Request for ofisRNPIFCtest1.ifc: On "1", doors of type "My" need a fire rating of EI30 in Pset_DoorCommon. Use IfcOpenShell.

First a look at what the model holds.

```python
import ifcopenshell
import ifcopenshell.util.element

model = ifcopenshell.open("ofisRNPIFCtest1.ifc")
print(model.schema)
storey = next(s for s in model.by_type("IfcBuildingStorey") if s.Name == "1")
doors = [e for e in ifcopenshell.util.element.get_decomposition(storey) if e.is_a("IfcDoor")]
seen = {}
for e in doors:
    element_type = ifcopenshell.util.element.get_type(e)
    key = (element_type.Name if element_type != e and element_type else None, ifcopenshell.util.element.get_pset(e, "Pset_DoorCommon", "FireRating"))
    seen[key] = seen.get(key, 0) + 1
for (name, value), count in sorted(seen.items(), key=str):
    print(count, "x", name, "|", value)
```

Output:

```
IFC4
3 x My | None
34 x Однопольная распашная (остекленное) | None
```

```python
import ifcopenshell
import ifcopenshell.api.pset
import ifcopenshell.util.element

model = ifcopenshell.open("ofisRNPIFCtest1.ifc")

storey = next(s for s in model.by_type("IfcBuildingStorey") if s.Name == "1")
doors = [e for e in ifcopenshell.util.element.get_decomposition(storey) if e.is_a("IfcDoor")]

count = 0
for e in doors:
    element_type = ifcopenshell.util.element.get_type(e)
    if element_type in (None, e) or element_type.Name != "My":
        continue
    # add_pset returns the element's existing set when there is one.
    pset = ifcopenshell.api.pset.add_pset(model, product=e, name="Pset_DoorCommon")
    ifcopenshell.api.pset.edit_pset(model, pset=pset, properties={"FireRating": "EI30"})
    count += 1

print(count, "doors updated")

model.write("ofisRNPIFCtest1_updated.ifc")
```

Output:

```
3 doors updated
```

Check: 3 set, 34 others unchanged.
